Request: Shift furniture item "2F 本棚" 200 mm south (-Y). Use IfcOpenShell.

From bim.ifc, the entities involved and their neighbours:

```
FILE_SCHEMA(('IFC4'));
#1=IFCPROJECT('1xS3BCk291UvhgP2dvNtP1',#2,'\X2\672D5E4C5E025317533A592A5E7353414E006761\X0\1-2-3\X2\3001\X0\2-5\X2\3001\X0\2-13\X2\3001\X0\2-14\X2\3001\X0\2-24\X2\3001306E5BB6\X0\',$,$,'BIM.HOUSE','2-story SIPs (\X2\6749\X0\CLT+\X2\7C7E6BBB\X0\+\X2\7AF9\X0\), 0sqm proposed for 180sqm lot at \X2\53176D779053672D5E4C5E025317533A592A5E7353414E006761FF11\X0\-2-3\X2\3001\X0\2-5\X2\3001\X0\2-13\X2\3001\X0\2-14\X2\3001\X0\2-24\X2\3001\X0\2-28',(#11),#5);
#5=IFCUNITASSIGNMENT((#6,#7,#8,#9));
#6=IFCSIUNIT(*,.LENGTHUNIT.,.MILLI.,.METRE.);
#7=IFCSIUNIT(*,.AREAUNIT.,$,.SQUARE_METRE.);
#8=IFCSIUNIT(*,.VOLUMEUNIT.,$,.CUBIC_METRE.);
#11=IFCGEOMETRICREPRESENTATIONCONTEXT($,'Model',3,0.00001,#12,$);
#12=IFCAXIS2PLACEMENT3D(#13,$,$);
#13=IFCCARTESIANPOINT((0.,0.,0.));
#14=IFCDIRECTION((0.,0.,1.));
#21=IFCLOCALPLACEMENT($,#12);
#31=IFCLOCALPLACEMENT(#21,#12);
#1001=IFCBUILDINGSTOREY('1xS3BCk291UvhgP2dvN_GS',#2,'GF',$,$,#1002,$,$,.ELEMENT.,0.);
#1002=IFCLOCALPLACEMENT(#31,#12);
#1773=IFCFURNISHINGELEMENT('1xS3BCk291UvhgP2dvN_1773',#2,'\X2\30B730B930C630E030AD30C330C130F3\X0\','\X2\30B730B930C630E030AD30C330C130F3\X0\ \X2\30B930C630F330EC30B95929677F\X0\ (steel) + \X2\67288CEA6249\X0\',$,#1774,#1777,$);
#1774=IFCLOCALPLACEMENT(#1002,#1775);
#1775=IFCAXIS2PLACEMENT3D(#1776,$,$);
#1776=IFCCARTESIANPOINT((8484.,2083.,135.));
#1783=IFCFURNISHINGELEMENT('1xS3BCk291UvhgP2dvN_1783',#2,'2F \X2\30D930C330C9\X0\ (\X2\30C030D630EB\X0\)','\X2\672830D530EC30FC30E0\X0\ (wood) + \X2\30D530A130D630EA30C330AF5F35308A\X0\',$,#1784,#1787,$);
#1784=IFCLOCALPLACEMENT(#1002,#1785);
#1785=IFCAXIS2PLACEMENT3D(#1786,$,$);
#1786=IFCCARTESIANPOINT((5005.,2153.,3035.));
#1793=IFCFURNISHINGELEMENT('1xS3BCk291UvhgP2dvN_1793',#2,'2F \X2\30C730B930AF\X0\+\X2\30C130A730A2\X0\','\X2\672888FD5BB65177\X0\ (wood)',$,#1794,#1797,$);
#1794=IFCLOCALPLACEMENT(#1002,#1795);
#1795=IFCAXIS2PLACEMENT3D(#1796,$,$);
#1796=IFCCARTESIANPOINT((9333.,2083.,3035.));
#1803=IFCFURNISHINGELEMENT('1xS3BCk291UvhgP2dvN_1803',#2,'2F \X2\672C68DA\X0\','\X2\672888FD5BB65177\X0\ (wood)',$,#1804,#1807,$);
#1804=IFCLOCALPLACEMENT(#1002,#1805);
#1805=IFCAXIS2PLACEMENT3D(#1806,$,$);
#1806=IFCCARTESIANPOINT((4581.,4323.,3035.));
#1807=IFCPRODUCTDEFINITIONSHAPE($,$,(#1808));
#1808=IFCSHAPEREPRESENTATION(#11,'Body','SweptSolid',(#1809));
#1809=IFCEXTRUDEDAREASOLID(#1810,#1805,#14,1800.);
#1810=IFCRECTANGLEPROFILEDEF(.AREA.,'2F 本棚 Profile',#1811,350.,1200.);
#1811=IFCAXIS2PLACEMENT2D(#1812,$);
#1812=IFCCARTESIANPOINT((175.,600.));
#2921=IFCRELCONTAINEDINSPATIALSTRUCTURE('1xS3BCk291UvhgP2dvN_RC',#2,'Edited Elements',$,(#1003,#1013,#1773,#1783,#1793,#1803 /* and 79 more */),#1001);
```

```python
import ifcopenshell
import ifcopenshell.api.geometry
import ifcopenshell.util.placement

model = ifcopenshell.open("bim.ifc")

item = model.by_id(1803)
matrix = ifcopenshell.util.placement.get_local_placement(item.ObjectPlacement)
matrix[1, 3] -= 200.0
ifcopenshell.api.geometry.edit_object_placement(model, product=item, matrix=matrix, is_si=False)

print(ifcopenshell.util.placement.get_local_placement(item.ObjectPlacement).round(3) + 0.0)

model.write("bim_edited.ifc")
```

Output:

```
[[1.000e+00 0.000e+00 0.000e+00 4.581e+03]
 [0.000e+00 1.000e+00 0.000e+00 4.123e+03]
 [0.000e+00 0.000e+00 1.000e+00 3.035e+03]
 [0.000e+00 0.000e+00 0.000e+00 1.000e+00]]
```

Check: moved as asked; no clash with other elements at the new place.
